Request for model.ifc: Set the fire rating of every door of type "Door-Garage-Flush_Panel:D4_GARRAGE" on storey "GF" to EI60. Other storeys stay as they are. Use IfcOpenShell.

First a look at what the model holds.

```python
import ifcopenshell
import ifcopenshell.util.element

model = ifcopenshell.open("model.ifc")
print(model.schema)
storey = next(s for s in model.by_type("IfcBuildingStorey") if s.Name == "GF")
doors = [e for e in ifcopenshell.util.element.get_decomposition(storey) if e.is_a("IfcDoor")]
seen = {}
for e in doors:
    element_type = ifcopenshell.util.element.get_type(e)
    key = (element_type.Name if element_type != e and element_type else None, ifcopenshell.util.element.get_pset(e, "Pset_DoorCommon", "FireRating"))
    seen[key] = seen.get(key, 0) + 1
for (name, value), count in sorted(seen.items(), key=str):
    print(count, "x", name, "|", value)
```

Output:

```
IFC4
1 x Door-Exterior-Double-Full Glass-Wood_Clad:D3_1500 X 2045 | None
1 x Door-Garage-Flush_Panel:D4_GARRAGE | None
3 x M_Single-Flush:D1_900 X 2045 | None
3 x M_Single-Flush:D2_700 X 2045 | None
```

```python
import ifcopenshell
import ifcopenshell.api.pset
import ifcopenshell.util.element

model = ifcopenshell.open("model.ifc")

storey = next(s for s in model.by_type("IfcBuildingStorey") if s.Name == "GF")
doors = [e for e in ifcopenshell.util.element.get_decomposition(storey) if e.is_a("IfcDoor")]

count = 0
for e in doors:
    element_type = ifcopenshell.util.element.get_type(e)
    if element_type in (None, e) or element_type.Name != "Door-Garage-Flush_Panel:D4_GARRAGE":
        continue
    # add_pset returns the element's existing set when there is one.
    pset = ifcopenshell.api.pset.add_pset(model, product=e, name="Pset_DoorCommon")
    ifcopenshell.api.pset.edit_pset(model, pset=pset, properties={"FireRating": "EI60"})
    count += 1

print(count, "doors updated")

model.write("model_rev.ifc")
```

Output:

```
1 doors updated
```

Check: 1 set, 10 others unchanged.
